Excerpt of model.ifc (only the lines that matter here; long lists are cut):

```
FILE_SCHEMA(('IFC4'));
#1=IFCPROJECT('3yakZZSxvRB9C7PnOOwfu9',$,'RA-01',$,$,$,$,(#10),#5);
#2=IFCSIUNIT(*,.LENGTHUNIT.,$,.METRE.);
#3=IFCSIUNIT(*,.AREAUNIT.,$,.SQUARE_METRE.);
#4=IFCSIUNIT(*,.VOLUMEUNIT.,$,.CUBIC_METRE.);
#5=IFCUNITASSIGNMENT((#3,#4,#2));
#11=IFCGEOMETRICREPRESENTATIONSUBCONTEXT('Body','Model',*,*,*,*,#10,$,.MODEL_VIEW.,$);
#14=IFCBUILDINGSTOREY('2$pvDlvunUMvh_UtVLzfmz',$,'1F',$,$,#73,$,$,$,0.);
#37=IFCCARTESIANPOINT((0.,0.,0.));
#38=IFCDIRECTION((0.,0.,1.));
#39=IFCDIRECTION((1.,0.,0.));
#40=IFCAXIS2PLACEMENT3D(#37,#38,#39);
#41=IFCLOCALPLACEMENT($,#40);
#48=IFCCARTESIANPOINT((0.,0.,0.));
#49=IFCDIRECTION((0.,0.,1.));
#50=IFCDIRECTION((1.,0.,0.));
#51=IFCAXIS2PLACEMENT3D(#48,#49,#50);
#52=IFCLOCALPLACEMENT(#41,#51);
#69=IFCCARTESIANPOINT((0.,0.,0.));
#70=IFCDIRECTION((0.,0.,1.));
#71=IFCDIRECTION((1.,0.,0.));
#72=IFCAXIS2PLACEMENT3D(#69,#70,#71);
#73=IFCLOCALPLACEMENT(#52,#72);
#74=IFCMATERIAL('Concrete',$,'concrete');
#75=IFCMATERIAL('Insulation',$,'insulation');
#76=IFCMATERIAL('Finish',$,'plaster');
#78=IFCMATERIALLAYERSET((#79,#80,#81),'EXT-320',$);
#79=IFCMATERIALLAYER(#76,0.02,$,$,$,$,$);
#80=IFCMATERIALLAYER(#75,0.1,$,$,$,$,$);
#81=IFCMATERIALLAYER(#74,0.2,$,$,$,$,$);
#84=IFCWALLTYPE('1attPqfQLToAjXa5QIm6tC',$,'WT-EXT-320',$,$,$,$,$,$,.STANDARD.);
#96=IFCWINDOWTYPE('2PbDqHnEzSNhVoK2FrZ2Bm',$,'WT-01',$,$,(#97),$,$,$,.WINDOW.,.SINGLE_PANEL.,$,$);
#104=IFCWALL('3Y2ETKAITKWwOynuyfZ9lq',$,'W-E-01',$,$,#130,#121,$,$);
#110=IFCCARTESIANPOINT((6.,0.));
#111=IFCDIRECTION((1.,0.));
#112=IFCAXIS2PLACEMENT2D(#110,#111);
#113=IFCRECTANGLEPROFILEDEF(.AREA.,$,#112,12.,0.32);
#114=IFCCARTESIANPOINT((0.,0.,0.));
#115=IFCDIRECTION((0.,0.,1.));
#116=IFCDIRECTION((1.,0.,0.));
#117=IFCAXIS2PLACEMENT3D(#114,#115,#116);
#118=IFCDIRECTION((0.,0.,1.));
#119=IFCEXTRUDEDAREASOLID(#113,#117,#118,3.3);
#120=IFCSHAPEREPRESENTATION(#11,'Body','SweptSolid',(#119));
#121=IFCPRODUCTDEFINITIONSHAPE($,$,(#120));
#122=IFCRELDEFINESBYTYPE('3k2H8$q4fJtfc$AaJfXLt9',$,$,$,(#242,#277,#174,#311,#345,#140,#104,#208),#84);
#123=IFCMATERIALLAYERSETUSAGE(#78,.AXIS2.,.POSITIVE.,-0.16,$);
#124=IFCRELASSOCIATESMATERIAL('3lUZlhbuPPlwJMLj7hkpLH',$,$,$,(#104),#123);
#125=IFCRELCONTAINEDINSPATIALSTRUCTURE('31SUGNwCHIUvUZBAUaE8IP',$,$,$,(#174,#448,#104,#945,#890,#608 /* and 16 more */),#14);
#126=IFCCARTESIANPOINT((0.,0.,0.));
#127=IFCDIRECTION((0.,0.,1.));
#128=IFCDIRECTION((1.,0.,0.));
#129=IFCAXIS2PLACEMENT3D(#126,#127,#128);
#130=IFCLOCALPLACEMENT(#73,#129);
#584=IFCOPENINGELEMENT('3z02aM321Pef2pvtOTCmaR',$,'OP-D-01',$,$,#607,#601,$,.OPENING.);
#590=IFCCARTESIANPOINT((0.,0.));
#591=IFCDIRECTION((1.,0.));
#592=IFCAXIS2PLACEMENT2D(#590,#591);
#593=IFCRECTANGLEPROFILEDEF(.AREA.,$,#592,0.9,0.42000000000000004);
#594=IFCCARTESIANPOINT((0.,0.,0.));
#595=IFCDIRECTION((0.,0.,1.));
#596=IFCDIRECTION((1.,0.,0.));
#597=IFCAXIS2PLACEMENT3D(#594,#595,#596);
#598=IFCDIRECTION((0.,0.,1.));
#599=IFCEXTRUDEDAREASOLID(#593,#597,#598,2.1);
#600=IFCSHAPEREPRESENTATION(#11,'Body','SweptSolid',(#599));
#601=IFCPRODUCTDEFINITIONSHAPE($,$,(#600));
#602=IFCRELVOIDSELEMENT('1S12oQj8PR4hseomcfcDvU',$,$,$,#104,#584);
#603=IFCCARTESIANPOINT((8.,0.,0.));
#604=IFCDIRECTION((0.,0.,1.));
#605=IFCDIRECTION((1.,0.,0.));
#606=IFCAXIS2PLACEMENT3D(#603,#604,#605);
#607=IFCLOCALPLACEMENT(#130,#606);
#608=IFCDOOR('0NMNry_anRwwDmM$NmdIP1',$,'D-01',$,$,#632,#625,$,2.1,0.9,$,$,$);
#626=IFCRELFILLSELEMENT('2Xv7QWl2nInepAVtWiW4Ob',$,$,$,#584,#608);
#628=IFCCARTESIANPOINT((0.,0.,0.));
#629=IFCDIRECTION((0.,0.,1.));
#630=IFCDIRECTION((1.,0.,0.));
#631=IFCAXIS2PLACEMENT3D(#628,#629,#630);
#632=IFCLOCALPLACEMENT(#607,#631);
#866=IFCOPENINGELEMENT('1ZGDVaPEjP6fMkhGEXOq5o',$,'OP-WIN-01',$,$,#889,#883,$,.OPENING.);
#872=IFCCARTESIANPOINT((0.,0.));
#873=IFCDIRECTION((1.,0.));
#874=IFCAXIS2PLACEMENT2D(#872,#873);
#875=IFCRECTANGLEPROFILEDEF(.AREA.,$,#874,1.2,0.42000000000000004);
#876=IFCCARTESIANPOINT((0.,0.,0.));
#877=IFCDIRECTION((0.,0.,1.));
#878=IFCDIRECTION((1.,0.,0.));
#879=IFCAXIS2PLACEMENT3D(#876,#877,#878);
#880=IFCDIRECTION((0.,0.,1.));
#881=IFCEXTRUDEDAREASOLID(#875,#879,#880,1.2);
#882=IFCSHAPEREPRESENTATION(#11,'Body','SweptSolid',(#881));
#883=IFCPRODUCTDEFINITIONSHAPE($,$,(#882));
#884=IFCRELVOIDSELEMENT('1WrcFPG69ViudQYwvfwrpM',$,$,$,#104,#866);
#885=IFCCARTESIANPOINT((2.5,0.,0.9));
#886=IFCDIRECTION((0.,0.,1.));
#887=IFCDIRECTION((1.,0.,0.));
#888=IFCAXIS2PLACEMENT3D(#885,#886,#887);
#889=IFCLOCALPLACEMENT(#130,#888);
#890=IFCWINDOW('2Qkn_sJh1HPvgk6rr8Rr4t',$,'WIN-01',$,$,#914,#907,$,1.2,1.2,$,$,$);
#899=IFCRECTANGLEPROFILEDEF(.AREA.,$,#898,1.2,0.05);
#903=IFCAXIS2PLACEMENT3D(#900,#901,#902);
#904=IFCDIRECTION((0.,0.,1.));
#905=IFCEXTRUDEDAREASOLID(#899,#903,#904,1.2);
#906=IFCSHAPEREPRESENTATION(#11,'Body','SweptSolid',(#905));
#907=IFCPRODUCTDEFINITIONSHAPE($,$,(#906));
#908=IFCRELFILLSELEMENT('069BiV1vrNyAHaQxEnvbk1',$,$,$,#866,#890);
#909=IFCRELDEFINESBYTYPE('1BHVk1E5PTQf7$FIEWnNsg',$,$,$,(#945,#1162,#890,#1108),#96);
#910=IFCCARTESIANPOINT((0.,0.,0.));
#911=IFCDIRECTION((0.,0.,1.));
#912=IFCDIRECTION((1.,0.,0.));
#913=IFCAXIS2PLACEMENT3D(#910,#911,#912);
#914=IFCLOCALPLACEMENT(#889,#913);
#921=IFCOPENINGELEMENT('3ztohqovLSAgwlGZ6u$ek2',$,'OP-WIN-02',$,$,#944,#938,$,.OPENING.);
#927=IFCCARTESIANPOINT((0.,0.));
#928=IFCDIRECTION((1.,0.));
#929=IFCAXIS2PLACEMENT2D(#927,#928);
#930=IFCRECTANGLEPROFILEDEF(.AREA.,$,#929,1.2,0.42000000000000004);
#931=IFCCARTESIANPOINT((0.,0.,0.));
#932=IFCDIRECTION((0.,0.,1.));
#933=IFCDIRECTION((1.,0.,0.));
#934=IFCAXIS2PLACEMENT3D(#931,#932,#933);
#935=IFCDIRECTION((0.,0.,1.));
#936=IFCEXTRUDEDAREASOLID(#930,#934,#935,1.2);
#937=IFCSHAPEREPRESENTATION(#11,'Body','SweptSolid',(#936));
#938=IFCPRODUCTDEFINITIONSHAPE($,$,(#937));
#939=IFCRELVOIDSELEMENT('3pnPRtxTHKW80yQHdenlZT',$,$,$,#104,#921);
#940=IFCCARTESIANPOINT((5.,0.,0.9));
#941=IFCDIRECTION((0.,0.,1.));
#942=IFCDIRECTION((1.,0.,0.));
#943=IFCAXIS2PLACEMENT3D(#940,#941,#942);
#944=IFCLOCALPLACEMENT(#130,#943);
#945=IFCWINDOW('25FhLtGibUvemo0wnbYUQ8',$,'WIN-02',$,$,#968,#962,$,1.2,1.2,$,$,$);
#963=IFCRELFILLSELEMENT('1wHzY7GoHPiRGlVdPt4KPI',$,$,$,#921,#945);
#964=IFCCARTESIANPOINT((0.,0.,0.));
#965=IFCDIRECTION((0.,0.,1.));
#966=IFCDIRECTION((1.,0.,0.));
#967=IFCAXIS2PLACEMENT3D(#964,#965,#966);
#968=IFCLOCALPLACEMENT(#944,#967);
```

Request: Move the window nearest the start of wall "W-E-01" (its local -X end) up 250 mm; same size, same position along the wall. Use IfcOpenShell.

```python
import numpy as np
import ifcopenshell
import ifcopenshell.api.geometry
import ifcopenshell.util.placement
import ifcopenshell.util.unit

model = ifcopenshell.open("model.ifc")
unit_scale = ifcopenshell.util.unit.calculate_unit_scale(model)

window = model.by_guid("2Qkn_sJh1HPvgk6rr8Rr4t")
opening = window.FillsVoids[0].RelatingOpeningElement
dz = 0.25 / unit_scale

shift = np.array([0.0, 0.0, dz])
# The window is placed relative to its opening, so it follows when the opening moves.
matrix = ifcopenshell.util.placement.get_local_placement(opening.ObjectPlacement)
matrix[:3, 3] += shift
ifcopenshell.api.geometry.edit_object_placement(
    model, product=opening, matrix=matrix, is_si=False, should_transform_children=True
)

print(f"moved by {dz * unit_scale:+.3f} m")

model.write("model_edited.ifc")
```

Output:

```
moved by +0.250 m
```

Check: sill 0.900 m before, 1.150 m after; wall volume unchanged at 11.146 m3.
